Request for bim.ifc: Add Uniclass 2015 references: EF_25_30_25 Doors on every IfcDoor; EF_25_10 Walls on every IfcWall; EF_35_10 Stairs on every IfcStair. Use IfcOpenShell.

First a look at what the model holds.

```python
import ifcopenshell

model = ifcopenshell.open("bim.ifc")
print(model.schema)
print("classifications:", [c.Name for c in model.by_type("IfcClassification")])
for ifc_class in ("IfcDoor", "IfcRoof", "IfcStair", "IfcWall", "IfcWindow"):
    print(ifc_class, len(model.by_type(ifc_class)))
```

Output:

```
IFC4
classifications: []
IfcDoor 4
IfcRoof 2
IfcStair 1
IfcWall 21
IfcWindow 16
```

```python
import ifcopenshell
import ifcopenshell.api.classification

model = ifcopenshell.open("bim.ifc")

system = ifcopenshell.api.classification.add_classification(model, classification="Uniclass 2015")

codes = {
    "IfcDoor": ("EF_25_30_25", "Doors"),
    "IfcWall": ("EF_25_10", "Walls"),
    "IfcStair": ("EF_35_10", "Stairs"),
}
for ifc_class, (code, name) in codes.items():
    products = model.by_type(ifc_class)
    ifcopenshell.api.classification.add_reference(
        model, products=products, classification=system, identification=code, name=name
    )
    print(code, len(products))

model.write("bim_edited.ifc")
```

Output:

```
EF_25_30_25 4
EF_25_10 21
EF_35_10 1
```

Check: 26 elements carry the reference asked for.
